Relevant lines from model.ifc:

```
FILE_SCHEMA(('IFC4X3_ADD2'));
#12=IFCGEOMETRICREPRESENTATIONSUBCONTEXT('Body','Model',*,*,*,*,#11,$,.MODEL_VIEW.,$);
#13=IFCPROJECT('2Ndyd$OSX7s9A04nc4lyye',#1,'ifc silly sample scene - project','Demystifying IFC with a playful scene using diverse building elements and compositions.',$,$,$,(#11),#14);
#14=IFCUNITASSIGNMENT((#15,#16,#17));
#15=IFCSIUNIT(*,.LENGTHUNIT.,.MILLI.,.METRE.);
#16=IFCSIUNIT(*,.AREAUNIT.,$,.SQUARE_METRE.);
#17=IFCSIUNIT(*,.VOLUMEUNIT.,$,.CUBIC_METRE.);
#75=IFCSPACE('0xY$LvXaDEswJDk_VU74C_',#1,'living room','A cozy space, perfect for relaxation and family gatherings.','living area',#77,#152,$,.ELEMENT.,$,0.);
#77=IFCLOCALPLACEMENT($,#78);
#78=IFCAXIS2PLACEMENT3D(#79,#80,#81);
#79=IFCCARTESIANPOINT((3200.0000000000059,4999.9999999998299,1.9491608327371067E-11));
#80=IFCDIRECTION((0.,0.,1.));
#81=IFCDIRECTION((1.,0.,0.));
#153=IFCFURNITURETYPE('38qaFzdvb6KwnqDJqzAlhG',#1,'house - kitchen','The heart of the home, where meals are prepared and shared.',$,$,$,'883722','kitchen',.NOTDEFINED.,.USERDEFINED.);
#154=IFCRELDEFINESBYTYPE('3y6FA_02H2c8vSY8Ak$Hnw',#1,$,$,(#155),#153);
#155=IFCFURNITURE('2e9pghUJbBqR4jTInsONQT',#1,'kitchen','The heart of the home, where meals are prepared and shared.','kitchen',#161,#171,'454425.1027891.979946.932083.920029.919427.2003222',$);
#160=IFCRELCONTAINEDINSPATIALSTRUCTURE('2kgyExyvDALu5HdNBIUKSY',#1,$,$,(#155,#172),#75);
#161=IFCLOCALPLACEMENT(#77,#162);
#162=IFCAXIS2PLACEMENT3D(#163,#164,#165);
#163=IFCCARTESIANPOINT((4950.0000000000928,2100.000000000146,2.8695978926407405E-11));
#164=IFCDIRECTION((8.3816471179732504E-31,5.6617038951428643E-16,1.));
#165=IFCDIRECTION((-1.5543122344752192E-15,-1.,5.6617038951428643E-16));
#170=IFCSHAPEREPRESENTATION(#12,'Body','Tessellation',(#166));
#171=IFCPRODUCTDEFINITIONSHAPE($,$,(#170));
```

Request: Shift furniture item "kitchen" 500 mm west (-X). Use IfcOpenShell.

```python
import ifcopenshell
import ifcopenshell.api.geometry
import ifcopenshell.util.placement
import ifcopenshell.util.unit

model = ifcopenshell.open("model.ifc")
unit_scale = ifcopenshell.util.unit.calculate_unit_scale(model)

item = model.by_guid("2e9pghUJbBqR4jTInsONQT")
matrix = ifcopenshell.util.placement.get_local_placement(item.ObjectPlacement)
matrix[0, 3] -= 0.5 / unit_scale
ifcopenshell.api.geometry.edit_object_placement(model, product=item, matrix=matrix, is_si=False)

print(ifcopenshell.util.placement.get_local_placement(item.ObjectPlacement).round(3) + 0.0)

model.write("model-out.ifc")
```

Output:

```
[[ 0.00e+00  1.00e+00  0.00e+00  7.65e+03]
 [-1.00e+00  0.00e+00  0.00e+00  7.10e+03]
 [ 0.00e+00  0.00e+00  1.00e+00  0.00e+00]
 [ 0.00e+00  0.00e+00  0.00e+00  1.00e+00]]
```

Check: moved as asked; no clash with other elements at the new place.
